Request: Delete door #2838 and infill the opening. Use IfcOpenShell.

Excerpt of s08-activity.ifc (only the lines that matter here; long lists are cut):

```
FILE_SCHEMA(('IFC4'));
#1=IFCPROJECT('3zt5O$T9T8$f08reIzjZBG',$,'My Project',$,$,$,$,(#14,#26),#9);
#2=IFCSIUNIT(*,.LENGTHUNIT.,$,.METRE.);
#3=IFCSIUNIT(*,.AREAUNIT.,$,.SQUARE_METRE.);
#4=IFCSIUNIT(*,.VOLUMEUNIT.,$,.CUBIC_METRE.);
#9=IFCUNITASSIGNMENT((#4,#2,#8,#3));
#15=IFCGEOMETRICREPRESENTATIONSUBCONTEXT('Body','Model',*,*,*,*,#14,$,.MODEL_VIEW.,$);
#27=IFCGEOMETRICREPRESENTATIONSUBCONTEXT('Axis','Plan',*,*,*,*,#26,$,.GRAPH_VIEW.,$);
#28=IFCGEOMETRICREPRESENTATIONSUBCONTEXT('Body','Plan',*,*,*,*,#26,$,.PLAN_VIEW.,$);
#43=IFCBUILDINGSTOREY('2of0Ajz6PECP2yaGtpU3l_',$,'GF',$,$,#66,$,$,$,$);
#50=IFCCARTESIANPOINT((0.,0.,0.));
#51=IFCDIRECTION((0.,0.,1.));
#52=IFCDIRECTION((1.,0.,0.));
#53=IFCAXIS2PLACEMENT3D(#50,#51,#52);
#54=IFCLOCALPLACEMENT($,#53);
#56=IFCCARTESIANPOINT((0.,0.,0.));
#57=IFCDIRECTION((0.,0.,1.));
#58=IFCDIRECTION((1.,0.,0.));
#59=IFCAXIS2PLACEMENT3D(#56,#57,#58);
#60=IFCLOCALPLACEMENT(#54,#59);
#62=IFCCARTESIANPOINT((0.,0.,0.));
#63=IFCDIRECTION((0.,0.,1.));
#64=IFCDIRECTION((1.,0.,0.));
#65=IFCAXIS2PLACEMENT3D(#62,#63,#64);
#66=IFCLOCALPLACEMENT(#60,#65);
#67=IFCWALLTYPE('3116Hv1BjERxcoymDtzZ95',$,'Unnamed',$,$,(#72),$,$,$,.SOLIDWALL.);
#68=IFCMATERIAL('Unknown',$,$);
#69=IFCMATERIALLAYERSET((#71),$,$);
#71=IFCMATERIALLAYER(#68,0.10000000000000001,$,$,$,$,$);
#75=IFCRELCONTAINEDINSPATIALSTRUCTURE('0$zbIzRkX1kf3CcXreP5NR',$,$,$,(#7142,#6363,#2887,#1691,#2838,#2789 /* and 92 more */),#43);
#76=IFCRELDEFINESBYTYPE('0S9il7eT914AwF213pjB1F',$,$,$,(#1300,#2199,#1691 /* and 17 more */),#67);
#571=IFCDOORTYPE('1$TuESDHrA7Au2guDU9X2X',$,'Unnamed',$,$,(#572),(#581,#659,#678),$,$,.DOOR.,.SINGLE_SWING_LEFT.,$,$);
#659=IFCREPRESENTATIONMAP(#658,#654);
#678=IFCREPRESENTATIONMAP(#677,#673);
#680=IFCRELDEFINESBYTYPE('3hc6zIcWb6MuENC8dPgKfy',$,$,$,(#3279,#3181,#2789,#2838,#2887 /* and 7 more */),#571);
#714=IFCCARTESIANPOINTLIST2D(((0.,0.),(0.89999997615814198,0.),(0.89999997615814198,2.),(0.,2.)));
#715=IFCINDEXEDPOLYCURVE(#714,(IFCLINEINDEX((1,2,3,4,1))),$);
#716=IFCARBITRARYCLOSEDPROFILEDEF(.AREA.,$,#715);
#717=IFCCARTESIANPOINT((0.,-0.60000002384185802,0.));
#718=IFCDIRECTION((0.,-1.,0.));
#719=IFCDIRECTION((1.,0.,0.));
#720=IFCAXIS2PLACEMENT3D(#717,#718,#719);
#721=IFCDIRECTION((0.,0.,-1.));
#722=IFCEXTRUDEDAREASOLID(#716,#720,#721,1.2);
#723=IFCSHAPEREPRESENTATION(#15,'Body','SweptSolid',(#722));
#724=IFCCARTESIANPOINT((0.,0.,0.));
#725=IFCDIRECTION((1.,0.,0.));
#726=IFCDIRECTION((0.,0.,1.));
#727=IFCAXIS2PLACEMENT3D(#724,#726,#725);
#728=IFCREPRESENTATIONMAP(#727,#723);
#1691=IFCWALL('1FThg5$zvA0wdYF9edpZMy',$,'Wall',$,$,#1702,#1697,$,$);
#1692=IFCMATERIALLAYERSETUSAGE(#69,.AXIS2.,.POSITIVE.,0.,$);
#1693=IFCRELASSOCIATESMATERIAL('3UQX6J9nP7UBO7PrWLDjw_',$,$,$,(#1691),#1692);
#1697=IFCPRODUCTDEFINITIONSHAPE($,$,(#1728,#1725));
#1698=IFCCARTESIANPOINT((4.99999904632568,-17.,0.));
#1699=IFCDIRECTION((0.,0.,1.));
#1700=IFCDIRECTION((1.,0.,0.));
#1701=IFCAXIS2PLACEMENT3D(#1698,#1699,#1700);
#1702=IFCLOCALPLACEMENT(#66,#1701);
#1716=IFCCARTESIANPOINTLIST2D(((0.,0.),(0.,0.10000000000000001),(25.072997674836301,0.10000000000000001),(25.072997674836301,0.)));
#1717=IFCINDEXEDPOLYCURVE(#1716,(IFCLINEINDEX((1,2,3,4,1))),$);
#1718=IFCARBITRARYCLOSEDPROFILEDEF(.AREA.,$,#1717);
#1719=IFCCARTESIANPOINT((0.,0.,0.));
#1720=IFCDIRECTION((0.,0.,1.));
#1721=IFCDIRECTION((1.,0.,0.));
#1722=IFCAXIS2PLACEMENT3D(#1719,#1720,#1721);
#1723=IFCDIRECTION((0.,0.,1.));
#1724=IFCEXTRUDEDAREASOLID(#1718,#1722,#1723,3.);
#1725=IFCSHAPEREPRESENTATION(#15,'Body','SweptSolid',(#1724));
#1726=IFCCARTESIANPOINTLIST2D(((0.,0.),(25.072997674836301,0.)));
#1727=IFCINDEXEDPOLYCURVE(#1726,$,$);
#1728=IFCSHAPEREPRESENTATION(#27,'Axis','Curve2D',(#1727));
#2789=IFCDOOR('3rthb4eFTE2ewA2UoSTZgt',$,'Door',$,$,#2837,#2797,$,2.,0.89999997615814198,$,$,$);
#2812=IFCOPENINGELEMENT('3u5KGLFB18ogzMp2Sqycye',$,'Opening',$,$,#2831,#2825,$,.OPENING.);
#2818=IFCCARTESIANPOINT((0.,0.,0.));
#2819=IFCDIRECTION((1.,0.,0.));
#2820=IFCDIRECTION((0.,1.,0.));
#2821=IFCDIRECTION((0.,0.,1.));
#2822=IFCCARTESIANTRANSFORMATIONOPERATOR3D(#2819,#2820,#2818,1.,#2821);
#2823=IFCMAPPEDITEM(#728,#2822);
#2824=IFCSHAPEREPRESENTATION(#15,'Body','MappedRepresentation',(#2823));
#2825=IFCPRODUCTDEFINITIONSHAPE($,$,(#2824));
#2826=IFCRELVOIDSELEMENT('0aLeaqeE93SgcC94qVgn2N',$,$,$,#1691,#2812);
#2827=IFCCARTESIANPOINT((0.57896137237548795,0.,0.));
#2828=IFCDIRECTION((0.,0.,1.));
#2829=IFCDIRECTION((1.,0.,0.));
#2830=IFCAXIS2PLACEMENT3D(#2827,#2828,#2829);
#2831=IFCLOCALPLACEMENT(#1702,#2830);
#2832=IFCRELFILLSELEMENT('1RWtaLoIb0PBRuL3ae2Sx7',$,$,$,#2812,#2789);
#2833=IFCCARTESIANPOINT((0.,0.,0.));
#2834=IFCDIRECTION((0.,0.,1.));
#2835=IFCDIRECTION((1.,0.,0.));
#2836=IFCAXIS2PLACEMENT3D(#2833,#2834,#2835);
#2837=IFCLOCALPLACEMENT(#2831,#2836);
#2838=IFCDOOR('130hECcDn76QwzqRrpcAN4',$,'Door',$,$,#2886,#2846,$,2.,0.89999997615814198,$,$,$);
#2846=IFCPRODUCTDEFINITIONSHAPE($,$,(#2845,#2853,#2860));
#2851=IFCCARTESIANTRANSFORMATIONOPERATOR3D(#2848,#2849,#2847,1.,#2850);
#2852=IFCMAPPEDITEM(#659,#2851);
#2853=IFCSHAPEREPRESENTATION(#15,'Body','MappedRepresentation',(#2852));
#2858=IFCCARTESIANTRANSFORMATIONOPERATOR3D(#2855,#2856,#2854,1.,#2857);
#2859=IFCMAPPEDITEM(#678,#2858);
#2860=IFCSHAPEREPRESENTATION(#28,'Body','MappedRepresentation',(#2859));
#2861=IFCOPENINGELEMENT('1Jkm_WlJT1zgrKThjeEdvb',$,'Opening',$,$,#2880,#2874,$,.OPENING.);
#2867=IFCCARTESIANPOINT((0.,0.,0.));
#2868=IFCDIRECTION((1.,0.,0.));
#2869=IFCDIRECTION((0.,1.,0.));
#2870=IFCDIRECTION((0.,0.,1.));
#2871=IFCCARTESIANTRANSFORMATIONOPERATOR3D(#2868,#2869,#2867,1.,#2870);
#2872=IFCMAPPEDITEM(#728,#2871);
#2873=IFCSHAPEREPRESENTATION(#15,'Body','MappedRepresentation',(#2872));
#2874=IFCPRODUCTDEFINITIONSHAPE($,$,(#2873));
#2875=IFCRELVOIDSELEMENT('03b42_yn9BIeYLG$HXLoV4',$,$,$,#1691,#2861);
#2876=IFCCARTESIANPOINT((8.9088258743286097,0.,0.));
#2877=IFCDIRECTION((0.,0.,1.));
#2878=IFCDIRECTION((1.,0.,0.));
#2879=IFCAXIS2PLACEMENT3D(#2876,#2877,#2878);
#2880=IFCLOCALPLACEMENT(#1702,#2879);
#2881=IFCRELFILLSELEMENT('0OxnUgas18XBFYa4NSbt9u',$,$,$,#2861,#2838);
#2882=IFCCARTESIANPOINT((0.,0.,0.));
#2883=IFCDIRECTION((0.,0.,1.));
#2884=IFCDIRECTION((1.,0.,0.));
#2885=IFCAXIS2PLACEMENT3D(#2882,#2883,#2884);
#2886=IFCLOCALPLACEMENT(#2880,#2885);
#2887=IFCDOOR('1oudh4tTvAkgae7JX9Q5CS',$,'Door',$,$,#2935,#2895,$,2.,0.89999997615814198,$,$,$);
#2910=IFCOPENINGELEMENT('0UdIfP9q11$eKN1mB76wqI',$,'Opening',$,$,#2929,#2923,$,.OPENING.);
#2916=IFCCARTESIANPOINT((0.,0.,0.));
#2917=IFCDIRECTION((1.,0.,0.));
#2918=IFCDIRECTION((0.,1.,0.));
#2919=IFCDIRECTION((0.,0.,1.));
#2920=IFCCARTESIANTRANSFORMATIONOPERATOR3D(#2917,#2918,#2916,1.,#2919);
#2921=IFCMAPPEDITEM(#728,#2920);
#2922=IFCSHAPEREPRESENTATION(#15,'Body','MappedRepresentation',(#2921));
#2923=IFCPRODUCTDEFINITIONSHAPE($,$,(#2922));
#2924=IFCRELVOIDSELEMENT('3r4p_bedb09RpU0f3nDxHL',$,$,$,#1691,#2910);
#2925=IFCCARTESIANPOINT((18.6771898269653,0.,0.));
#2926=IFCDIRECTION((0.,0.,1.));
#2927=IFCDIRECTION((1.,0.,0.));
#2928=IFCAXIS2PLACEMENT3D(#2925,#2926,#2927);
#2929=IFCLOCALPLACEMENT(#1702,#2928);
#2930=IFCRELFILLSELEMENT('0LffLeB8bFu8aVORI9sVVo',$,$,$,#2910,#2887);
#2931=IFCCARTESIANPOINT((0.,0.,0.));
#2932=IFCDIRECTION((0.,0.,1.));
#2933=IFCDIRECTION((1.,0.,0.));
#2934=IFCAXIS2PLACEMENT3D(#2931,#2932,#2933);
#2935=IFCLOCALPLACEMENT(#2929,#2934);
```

```python
import ifcopenshell
import ifcopenshell.api.feature
import ifcopenshell.api.root
import ifcopenshell.geom
import ifcopenshell.util.shape

model = ifcopenshell.open("s08-activity.ifc")
settings = ifcopenshell.geom.settings()


def volume(element):
    """Net volume in cubic metres, openings subtracted."""
    shape = ifcopenshell.geom.create_shape(settings, element)
    return ifcopenshell.util.shape.get_volume(shape.geometry)


door = model.by_id(2838)
opening = door.FillsVoids[0].RelatingOpeningElement
wall = opening.VoidsElements[0].RelatingBuildingElement
before = volume(wall)

ifcopenshell.api.root.remove_product(model, product=door)
ifcopenshell.api.feature.remove_feature(model, feature=opening)

after = volume(wall)

print(f"wall volume {before:.3f} -> {after:.3f} m3")

model.write("s08-activity_edited.ifc")
```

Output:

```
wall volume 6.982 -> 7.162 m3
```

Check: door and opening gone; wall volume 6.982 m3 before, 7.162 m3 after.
